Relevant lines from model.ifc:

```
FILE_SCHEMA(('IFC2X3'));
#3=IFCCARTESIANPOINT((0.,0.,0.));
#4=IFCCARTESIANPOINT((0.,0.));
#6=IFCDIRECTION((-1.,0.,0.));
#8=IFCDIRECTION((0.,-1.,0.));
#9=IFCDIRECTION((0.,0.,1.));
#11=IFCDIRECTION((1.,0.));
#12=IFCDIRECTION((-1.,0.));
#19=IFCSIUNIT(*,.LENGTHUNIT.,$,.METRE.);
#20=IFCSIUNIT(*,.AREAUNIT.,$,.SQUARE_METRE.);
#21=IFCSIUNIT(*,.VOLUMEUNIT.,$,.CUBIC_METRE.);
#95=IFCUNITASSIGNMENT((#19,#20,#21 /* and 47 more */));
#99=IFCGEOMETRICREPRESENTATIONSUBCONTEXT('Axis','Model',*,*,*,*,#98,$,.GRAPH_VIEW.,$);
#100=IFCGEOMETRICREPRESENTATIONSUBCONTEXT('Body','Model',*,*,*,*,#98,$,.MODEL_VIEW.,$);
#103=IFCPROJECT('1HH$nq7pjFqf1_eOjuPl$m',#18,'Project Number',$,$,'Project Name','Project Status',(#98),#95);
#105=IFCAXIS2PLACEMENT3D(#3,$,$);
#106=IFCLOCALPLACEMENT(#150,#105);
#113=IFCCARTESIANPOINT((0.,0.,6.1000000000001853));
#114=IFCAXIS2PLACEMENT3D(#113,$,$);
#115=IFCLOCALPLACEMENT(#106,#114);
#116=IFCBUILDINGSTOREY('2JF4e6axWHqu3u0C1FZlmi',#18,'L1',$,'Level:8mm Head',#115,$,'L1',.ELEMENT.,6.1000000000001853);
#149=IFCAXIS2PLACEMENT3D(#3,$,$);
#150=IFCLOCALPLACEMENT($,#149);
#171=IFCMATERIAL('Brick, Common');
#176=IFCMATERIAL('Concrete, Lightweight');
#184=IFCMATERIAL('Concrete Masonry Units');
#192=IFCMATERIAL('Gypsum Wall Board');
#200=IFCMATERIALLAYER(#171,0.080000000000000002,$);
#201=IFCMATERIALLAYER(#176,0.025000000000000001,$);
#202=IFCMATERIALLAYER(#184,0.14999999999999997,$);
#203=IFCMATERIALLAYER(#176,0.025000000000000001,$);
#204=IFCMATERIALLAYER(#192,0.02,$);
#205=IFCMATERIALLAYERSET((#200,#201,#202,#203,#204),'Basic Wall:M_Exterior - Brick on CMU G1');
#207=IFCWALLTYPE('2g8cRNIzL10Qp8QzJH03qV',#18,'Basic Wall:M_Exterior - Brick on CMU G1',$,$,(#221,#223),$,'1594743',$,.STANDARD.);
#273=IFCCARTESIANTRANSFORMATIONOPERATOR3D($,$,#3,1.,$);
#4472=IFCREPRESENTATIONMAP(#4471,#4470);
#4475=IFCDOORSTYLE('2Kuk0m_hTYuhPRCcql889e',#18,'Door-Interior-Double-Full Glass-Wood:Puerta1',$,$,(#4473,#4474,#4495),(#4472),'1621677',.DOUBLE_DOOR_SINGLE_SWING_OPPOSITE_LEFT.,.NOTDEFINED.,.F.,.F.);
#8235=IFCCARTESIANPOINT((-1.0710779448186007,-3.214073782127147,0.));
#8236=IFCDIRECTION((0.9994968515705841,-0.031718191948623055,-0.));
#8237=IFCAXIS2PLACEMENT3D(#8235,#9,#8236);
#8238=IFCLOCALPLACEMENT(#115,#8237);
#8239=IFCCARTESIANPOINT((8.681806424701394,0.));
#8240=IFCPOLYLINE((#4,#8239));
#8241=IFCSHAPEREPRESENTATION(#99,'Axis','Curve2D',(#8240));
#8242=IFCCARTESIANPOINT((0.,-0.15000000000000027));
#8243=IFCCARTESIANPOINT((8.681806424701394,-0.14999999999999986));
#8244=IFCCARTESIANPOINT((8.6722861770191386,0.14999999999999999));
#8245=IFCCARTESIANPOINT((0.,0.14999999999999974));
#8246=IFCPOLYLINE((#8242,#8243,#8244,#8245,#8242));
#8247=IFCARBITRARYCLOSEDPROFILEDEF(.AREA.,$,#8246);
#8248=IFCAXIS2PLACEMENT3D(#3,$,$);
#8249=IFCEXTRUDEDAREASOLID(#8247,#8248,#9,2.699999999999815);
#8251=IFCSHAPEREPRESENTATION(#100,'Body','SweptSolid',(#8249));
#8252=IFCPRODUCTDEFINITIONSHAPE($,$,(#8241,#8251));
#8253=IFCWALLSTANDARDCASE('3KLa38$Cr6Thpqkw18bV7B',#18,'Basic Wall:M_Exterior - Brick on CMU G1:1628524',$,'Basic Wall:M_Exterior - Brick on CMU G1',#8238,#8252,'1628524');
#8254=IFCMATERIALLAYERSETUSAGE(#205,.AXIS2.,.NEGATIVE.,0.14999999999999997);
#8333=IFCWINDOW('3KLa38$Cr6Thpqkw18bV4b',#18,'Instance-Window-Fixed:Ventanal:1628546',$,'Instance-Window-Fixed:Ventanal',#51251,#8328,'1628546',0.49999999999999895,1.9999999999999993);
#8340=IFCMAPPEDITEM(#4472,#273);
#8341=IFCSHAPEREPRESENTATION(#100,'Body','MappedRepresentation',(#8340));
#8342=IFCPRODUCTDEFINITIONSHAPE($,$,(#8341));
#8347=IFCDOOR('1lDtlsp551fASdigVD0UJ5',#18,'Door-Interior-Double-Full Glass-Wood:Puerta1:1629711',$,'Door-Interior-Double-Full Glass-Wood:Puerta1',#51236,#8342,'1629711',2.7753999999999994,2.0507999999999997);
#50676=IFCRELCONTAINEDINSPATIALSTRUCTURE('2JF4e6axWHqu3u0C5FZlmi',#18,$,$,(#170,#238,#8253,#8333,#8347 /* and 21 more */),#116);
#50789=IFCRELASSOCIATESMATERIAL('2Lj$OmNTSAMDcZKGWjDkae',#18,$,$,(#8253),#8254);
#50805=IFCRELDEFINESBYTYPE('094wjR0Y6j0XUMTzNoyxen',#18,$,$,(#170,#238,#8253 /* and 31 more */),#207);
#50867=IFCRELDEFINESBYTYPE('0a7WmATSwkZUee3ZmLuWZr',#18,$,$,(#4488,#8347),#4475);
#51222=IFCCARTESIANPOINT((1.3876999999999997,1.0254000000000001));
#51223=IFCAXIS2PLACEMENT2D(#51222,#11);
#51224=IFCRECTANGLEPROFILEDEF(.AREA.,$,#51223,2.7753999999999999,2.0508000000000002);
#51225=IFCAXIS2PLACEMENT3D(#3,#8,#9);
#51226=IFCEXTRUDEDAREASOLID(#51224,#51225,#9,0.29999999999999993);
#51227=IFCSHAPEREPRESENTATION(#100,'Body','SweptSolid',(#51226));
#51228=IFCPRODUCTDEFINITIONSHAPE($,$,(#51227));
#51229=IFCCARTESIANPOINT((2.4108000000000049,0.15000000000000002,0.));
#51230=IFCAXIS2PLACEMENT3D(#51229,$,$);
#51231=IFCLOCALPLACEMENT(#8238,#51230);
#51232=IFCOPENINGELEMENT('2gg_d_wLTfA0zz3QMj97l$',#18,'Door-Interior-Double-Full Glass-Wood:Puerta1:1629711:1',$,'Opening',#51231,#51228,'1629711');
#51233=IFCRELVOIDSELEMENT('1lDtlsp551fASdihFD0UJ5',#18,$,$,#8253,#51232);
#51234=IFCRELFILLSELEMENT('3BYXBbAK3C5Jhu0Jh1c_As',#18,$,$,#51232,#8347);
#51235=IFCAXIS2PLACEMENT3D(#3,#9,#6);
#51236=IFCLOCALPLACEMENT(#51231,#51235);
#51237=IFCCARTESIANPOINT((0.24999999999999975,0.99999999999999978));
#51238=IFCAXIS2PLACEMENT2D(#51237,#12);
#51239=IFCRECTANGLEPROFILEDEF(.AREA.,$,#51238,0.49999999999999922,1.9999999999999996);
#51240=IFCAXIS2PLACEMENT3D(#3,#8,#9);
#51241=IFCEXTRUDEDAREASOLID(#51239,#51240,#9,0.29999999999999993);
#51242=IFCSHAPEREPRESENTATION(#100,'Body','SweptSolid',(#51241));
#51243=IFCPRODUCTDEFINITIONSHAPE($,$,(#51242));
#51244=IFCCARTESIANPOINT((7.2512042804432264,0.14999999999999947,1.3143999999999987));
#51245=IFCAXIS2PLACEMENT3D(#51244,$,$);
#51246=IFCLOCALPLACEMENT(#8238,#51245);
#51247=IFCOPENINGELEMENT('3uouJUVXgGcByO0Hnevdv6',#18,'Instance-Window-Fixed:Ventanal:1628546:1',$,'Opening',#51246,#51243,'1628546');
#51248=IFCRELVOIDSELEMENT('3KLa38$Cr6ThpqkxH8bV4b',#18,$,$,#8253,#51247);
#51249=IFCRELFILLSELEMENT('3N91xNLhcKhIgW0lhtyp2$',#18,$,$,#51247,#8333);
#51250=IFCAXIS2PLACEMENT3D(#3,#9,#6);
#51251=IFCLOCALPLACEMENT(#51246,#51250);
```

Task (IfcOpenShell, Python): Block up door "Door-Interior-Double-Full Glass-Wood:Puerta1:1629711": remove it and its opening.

```python
import ifcopenshell
import ifcopenshell.api.feature
import ifcopenshell.api.root
import ifcopenshell.geom
import ifcopenshell.util.shape

model = ifcopenshell.open("model.ifc")
settings = ifcopenshell.geom.settings()


def volume(element):
    """Net volume in cubic metres, openings subtracted."""
    shape = ifcopenshell.geom.create_shape(settings, element)
    return ifcopenshell.util.shape.get_volume(shape.geometry)


door = model.by_guid("1lDtlsp551fASdigVD0UJ5")
opening = door.FillsVoids[0].RelatingOpeningElement
wall = opening.VoidsElements[0].RelatingBuildingElement
before = volume(wall)

ifcopenshell.api.root.remove_product(model, product=door)
ifcopenshell.api.feature.remove_feature(model, feature=opening)

after = volume(wall)

print(f"wall volume {before:.3f} -> {after:.3f} m3")

model.write("model_updated.ifc")
```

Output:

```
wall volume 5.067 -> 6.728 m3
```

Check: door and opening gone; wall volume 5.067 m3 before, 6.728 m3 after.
